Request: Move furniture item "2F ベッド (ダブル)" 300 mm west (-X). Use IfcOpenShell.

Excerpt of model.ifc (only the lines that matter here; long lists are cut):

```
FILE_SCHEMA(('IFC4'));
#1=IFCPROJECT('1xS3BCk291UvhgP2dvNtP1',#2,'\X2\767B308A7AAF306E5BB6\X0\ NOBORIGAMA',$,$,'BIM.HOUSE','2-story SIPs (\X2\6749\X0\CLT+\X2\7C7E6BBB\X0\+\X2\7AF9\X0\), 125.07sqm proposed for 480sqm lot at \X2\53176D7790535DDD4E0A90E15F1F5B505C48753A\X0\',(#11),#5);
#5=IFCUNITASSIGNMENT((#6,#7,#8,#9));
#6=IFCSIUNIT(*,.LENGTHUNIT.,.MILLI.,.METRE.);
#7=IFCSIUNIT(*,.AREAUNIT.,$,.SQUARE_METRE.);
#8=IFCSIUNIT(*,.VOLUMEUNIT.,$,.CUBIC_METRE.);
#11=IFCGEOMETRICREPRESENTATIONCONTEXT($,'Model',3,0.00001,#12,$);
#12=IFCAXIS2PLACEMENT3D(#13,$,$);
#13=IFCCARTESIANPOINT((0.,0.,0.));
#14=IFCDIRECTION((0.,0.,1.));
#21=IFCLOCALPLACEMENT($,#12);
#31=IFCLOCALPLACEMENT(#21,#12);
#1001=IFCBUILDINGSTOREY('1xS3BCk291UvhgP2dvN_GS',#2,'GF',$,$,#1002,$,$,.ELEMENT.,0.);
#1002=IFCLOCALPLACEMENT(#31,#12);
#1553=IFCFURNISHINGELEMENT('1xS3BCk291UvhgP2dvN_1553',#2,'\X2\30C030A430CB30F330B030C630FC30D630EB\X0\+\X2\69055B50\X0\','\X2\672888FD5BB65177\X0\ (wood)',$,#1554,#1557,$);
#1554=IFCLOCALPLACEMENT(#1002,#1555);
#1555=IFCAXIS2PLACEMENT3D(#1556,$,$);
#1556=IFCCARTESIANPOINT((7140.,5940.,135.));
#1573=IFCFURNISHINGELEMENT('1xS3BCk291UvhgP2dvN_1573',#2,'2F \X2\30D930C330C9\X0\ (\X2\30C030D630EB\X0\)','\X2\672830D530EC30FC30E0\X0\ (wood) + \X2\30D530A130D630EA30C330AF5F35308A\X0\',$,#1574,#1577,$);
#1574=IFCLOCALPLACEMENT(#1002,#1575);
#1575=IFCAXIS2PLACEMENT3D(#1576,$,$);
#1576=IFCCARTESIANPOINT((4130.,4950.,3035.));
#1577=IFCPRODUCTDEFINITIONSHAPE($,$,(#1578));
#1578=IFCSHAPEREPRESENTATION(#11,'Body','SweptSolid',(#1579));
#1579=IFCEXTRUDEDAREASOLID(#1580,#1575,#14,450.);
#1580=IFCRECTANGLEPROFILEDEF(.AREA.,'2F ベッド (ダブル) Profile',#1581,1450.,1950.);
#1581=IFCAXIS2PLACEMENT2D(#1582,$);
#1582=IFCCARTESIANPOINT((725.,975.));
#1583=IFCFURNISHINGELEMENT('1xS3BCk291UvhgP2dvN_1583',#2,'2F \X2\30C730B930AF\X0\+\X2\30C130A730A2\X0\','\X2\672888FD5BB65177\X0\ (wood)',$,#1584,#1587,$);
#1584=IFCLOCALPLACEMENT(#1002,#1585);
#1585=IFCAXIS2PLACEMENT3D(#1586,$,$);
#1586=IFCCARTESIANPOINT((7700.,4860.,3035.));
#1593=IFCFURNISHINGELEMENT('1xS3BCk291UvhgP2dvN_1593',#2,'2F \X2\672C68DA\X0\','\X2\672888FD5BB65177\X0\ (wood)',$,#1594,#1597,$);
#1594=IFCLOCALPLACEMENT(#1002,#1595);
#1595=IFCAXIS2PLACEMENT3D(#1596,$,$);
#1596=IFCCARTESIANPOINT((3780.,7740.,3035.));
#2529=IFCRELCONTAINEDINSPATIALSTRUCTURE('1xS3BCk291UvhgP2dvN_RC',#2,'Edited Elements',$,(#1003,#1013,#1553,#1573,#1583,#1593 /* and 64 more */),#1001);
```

```python
import ifcopenshell
import ifcopenshell.api.geometry
import ifcopenshell.util.placement
import ifcopenshell.util.unit

model = ifcopenshell.open("model.ifc")
unit_scale = ifcopenshell.util.unit.calculate_unit_scale(model)

item = model.by_guid("1xS3BCk291UvhgP2dvN_1573")
matrix = ifcopenshell.util.placement.get_local_placement(item.ObjectPlacement)
matrix[0, 3] -= 0.3 / unit_scale
ifcopenshell.api.geometry.edit_object_placement(model, product=item, matrix=matrix, is_si=False)

print(ifcopenshell.util.placement.get_local_placement(item.ObjectPlacement).round(3) + 0.0)

model.write("model_edited.ifc")
```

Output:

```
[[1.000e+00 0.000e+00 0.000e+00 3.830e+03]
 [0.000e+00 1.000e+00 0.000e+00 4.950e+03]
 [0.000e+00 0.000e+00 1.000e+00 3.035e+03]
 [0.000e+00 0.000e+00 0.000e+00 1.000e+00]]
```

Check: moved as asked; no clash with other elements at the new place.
